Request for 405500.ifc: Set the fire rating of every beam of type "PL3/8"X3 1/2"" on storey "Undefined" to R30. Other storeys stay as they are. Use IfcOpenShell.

First a look at what the model holds.

```python
import ifcopenshell
import ifcopenshell.util.element

model = ifcopenshell.open("405500.ifc")
print(model.schema)
storey = next(s for s in model.by_type("IfcBuildingStorey") if s.Name == "Undefined")
beams = [e for e in ifcopenshell.util.element.get_decomposition(storey) if e.is_a("IfcBeam")]
seen = {}
for e in beams:
    element_type = ifcopenshell.util.element.get_type(e)
    key = (element_type.Name if element_type != e and element_type else None, ifcopenshell.util.element.get_pset(e, "Pset_BeamCommon", "FireRating"))
    seen[key] = seen.get(key, 0) + 1
for (name, value), count in sorted(seen.items(), key=str):
    print(count, "x", name, "|", value)
```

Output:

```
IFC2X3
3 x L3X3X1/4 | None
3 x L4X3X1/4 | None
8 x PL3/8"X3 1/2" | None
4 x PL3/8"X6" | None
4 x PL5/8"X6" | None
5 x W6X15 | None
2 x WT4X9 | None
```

```python
import ifcopenshell
import ifcopenshell.api.pset
import ifcopenshell.util.element

model = ifcopenshell.open("405500.ifc")

storey = next(s for s in model.by_type("IfcBuildingStorey") if s.Name == "Undefined")
beams = [e for e in ifcopenshell.util.element.get_decomposition(storey) if e.is_a("IfcBeam")]

count = 0
for e in beams:
    element_type = ifcopenshell.util.element.get_type(e)
    if element_type in (None, e) or element_type.Name != 'PL3/8"X3 1/2"':
        continue
    found = ifcopenshell.util.element.get_pset(e, "Pset_BeamCommon", should_inherit=False)
    if found:
        pset = model.by_id(found["id"])
        if len(ifcopenshell.util.element.get_elements_by_pset(pset)) > 1:
            pset = ifcopenshell.api.pset.unshare_pset(model, products=[e], pset=pset)[0]
    else:
        pset = ifcopenshell.api.pset.add_pset(model, product=e, name="Pset_BeamCommon")
    ifcopenshell.api.pset.edit_pset(model, pset=pset, properties={"FireRating": "R30"})
    count += 1

print(count, "beams updated")

model.write("405500-out.ifc")
```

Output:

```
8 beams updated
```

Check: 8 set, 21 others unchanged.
